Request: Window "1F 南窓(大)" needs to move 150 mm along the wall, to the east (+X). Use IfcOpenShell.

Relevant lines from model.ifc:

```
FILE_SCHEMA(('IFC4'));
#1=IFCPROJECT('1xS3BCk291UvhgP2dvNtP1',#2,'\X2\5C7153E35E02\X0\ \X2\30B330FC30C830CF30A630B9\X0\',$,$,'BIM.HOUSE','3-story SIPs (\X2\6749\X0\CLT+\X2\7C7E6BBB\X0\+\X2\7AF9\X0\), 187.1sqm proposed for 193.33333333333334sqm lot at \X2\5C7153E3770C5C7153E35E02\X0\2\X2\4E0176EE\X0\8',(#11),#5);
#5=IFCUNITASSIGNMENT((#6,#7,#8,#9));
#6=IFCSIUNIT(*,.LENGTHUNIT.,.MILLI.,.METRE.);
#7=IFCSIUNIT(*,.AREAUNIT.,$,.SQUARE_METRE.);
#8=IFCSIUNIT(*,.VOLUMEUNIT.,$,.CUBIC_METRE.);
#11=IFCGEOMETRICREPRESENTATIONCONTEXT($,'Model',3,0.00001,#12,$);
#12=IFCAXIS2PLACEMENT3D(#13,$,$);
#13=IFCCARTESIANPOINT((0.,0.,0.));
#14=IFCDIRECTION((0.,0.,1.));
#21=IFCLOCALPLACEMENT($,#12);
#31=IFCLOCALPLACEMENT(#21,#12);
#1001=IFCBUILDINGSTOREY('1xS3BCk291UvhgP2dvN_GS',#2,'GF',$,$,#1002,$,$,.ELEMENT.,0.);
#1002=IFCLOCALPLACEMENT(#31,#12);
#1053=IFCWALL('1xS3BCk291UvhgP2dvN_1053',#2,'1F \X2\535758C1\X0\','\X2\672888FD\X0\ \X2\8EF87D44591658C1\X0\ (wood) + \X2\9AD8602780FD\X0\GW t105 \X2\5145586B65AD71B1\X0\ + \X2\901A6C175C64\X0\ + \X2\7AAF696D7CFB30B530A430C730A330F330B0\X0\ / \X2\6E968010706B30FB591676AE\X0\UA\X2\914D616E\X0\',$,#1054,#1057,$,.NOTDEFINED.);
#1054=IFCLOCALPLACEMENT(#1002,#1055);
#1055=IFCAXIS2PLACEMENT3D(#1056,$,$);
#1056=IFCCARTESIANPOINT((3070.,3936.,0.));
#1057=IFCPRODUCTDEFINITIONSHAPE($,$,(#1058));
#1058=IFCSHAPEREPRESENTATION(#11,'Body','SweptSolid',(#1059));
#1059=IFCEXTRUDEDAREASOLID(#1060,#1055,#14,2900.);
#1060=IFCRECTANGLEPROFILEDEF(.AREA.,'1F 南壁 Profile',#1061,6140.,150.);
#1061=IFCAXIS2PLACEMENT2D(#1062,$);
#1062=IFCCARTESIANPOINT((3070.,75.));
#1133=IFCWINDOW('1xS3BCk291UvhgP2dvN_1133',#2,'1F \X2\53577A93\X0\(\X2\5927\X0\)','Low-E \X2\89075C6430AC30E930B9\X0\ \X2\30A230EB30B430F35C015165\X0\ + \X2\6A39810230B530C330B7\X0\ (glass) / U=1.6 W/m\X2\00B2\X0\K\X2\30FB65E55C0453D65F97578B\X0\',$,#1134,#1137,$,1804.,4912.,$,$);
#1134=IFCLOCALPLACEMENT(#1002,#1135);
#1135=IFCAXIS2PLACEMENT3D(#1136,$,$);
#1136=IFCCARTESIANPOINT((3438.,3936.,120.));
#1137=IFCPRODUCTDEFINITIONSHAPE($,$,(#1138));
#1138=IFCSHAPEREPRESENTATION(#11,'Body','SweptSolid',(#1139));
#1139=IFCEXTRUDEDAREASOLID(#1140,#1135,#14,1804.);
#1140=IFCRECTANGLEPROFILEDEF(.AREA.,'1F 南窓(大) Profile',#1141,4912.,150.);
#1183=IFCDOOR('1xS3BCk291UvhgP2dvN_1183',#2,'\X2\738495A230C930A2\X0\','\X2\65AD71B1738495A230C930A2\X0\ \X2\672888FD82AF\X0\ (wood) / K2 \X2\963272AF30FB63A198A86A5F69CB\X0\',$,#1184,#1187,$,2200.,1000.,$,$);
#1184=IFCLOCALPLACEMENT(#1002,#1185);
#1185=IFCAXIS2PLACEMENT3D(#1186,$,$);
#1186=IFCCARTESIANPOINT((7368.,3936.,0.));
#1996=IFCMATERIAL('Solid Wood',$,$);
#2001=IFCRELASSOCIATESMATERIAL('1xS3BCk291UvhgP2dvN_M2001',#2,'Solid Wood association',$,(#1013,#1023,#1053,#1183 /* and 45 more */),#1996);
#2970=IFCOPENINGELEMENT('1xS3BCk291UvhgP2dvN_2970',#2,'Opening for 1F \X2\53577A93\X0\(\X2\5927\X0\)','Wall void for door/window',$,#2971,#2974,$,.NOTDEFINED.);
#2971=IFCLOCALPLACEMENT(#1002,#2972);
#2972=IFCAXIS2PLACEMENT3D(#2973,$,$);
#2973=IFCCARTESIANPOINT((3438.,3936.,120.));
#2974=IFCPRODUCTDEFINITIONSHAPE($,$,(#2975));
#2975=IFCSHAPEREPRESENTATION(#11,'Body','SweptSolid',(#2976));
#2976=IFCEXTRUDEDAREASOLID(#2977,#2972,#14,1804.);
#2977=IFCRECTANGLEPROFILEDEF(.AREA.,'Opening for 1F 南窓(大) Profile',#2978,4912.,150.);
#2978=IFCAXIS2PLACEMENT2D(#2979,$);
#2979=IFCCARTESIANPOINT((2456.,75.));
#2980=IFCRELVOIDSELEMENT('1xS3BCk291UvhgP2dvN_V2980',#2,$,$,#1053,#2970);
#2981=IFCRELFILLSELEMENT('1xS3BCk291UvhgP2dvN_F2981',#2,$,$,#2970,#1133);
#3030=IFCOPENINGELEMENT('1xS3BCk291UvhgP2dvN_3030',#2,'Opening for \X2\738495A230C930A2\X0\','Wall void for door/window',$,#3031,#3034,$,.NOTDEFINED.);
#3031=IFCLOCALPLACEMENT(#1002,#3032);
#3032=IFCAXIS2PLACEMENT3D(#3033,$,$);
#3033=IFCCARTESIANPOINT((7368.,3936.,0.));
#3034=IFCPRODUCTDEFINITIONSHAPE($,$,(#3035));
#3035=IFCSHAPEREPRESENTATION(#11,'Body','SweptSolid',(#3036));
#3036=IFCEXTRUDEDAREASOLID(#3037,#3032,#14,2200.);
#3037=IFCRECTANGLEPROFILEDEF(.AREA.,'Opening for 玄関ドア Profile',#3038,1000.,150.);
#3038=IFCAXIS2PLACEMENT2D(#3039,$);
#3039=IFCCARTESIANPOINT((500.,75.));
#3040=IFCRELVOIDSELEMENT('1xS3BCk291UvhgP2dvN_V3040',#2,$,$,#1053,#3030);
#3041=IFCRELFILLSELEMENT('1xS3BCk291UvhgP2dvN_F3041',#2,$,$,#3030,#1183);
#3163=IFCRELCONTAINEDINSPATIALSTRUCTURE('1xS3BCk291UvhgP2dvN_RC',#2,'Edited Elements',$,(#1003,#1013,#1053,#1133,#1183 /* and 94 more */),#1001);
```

```python
import ifcopenshell
import ifcopenshell.api.geometry
import ifcopenshell.util.placement

model = ifcopenshell.open("model.ifc")

window = model.by_guid("1xS3BCk291UvhgP2dvN_1133")
opening = window.FillsVoids[0].RelatingOpeningElement
wall = opening.VoidsElements[0].RelatingBuildingElement

wall_matrix = ifcopenshell.util.placement.get_local_placement(wall.ObjectPlacement)
shift = wall_matrix[:3, 0] * 150.0
before = ifcopenshell.util.placement.get_local_placement(window.ObjectPlacement)[:3, 3].copy()

# The window is not placed relative to its opening, so move both.
for product in (opening, window):
    matrix = ifcopenshell.util.placement.get_local_placement(product.ObjectPlacement)
    matrix[:3, 3] += shift
    ifcopenshell.api.geometry.edit_object_placement(model, product=product, matrix=matrix, is_si=False)

after = ifcopenshell.util.placement.get_local_placement(window.ObjectPlacement)[:3, 3]
print("window moved by", (after - before).round(3) + 0.0)

model.write("model_v2.ifc")
```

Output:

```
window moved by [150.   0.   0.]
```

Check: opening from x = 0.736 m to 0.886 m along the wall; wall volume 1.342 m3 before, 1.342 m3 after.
